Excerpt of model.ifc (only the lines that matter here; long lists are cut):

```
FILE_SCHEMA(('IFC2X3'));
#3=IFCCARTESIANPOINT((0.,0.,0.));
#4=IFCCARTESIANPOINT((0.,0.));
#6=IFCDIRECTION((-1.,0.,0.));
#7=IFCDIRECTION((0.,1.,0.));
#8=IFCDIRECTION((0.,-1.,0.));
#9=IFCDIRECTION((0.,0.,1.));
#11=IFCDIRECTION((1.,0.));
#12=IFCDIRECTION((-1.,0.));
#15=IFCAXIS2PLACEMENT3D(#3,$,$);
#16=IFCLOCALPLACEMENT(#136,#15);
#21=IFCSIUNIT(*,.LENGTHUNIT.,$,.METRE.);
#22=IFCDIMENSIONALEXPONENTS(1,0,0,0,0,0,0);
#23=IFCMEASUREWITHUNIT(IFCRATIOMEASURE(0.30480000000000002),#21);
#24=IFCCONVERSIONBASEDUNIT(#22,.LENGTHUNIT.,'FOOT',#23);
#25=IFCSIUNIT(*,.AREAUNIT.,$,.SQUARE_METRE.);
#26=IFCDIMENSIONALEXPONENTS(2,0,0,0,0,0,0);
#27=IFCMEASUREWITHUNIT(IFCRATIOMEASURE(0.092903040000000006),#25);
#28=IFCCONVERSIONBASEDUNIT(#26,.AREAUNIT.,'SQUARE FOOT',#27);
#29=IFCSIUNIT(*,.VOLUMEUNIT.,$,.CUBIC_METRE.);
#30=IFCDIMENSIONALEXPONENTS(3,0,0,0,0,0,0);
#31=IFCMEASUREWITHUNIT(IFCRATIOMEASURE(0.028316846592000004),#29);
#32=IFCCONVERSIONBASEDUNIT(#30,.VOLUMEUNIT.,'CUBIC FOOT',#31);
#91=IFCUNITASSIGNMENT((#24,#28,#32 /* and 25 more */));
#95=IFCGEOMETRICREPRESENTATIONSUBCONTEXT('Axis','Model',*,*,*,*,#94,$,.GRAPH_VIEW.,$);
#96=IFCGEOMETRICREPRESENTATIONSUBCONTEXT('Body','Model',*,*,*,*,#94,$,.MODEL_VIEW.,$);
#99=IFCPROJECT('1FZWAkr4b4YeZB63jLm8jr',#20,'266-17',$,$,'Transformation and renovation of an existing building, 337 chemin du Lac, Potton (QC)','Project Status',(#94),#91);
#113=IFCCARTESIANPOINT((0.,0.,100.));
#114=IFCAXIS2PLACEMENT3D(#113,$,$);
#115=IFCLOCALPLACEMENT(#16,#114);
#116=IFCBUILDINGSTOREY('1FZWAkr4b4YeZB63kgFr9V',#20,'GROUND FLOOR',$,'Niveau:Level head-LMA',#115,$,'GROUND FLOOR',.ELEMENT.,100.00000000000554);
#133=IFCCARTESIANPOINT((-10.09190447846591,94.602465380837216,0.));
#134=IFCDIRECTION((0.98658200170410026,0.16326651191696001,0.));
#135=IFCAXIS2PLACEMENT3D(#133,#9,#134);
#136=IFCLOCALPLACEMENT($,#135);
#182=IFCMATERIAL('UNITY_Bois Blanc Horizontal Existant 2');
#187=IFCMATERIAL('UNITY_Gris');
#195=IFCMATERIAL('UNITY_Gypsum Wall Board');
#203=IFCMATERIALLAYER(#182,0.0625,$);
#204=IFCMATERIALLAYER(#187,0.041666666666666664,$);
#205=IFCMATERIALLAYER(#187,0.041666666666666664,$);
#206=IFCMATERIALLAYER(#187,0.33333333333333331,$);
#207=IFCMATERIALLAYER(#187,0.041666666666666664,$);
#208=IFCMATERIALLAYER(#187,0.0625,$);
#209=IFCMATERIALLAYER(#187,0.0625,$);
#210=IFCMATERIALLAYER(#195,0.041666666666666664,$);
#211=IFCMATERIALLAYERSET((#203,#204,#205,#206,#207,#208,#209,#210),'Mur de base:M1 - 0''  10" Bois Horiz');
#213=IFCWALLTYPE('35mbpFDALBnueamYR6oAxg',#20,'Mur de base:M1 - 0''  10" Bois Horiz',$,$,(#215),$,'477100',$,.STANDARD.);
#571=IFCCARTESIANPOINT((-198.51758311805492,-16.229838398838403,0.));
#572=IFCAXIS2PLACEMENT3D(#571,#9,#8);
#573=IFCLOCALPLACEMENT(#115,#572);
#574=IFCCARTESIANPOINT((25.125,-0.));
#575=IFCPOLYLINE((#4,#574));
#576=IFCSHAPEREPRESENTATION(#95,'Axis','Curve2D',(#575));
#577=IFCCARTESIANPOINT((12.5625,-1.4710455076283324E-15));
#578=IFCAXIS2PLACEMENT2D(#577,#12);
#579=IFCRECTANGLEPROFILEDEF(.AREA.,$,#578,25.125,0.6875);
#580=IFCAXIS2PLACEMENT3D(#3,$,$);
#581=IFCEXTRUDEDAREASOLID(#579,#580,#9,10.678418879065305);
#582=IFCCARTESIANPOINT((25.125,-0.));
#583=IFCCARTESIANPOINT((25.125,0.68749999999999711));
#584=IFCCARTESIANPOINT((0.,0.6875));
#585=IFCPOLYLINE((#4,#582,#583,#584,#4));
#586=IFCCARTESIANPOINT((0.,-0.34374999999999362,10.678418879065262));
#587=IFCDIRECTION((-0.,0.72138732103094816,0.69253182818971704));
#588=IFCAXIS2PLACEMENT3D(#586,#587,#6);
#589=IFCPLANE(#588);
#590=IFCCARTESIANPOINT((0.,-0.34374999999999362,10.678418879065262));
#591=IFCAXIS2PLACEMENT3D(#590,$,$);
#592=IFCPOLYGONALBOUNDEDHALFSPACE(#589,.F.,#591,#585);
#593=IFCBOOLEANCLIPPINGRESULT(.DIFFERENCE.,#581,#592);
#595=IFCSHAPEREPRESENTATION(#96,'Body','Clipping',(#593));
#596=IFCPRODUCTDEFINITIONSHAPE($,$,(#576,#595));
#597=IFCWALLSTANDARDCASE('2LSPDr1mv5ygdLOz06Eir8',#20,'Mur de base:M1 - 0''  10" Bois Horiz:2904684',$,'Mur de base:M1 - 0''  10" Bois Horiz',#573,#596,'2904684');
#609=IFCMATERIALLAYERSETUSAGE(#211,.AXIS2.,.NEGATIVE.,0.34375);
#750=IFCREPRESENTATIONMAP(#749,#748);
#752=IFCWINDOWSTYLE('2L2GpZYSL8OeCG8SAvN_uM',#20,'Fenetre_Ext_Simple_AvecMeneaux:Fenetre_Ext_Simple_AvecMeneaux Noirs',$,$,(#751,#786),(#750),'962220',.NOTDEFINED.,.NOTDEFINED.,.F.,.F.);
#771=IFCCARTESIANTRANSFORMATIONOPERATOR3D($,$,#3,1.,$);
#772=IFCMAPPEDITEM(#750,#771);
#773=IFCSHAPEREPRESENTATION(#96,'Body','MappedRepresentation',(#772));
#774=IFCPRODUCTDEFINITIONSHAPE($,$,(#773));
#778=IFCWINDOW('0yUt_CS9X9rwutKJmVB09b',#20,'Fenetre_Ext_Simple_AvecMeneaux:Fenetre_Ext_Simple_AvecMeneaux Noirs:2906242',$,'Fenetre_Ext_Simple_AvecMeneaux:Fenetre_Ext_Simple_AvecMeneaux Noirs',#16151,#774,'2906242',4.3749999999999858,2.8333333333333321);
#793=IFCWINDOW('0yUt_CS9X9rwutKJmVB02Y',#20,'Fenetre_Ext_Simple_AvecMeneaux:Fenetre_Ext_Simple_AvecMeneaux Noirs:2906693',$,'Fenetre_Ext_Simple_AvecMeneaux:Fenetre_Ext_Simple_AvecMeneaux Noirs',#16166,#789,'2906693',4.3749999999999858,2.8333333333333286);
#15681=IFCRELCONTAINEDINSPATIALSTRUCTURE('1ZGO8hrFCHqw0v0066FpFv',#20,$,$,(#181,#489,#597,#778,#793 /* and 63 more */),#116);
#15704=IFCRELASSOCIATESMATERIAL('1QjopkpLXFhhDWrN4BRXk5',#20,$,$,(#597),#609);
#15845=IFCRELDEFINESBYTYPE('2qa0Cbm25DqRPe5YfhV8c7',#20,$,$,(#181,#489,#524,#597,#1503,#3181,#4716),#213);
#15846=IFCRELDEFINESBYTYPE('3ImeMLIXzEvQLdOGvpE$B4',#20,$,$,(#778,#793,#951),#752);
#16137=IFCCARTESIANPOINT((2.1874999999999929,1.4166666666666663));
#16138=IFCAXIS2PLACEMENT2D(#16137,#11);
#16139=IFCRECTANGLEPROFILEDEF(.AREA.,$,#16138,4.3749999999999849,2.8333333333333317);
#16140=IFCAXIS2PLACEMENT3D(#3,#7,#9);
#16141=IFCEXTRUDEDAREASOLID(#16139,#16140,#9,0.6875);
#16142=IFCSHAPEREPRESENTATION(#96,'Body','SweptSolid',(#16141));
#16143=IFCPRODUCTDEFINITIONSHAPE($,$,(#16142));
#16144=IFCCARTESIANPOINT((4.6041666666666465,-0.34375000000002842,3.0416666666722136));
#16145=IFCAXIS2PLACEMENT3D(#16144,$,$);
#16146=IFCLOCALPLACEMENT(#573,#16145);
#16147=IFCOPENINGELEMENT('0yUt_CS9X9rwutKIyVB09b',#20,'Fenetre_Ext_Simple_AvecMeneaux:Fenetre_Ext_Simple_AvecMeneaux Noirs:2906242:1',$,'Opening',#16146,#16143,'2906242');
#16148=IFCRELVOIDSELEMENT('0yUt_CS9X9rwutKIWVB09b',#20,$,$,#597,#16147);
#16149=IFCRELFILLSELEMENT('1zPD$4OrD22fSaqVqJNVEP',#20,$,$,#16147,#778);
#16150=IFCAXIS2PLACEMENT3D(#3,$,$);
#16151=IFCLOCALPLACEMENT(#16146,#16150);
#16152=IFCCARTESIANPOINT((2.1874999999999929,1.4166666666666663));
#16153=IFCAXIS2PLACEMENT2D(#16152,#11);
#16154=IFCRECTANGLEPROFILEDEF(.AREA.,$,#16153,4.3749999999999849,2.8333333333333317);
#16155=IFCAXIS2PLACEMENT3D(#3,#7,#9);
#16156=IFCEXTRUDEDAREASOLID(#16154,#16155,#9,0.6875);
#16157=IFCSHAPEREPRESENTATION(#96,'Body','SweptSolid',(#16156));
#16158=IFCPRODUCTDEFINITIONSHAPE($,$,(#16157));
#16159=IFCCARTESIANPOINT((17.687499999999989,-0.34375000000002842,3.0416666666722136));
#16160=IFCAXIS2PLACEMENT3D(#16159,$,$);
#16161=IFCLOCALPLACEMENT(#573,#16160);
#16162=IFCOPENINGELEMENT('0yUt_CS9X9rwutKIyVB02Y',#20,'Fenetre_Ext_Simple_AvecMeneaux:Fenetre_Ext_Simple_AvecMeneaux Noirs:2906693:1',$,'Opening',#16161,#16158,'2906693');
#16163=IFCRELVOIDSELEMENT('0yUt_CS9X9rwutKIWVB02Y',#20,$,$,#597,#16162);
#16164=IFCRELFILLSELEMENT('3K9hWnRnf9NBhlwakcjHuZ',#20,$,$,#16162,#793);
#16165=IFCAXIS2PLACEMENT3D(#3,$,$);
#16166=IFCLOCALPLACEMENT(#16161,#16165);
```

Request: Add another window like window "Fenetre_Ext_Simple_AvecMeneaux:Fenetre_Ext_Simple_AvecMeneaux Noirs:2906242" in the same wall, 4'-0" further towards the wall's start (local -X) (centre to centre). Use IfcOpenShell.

```python
import ifcopenshell
import ifcopenshell.api.feature
import ifcopenshell.api.geometry
import ifcopenshell.api.root
import ifcopenshell.geom
import ifcopenshell.util.element
import ifcopenshell.util.placement
import ifcopenshell.util.shape
import ifcopenshell.util.unit

model = ifcopenshell.open("model.ifc")
unit_scale = ifcopenshell.util.unit.calculate_unit_scale(model)
settings = ifcopenshell.geom.settings()


def volume(element):
    """Net volume in cubic metres, openings subtracted."""
    shape = ifcopenshell.geom.create_shape(settings, element)
    return ifcopenshell.util.shape.get_volume(shape.geometry)


def reuse_history(source, copy):
    """copy_class also copies each property set's owner history, people and application; keep the originals."""
    for rel in copy.IsDefinedBy:
        if rel.is_a("IfcRelDefinesByProperties") and (history := rel.RelatingPropertyDefinition.OwnerHistory):
            rel.RelatingPropertyDefinition.OwnerHistory = source.OwnerHistory
            ifcopenshell.util.element.remove_deep2(model, history)


window = model.by_guid("0yUt_CS9X9rwutKJmVB09b")
opening = window.FillsVoids[0].RelatingOpeningElement
wall = opening.VoidsElements[0].RelatingBuildingElement
before = volume(wall)
shift = ifcopenshell.util.placement.get_local_placement(wall.ObjectPlacement)[:3, 0] * -48 * 0.0254 / unit_scale

# copy_class copies the void relationship, type, container and properties, but no geometry.
new_opening = ifcopenshell.api.root.copy_class(model, product=opening)
new_opening.Representation = ifcopenshell.util.element.copy_deep(
    model, opening.Representation, exclude=["IfcGeometricRepresentationContext", "IfcRepresentationMap"]
)
new_opening.Name = "Fenetre_Ext_Simple_AvecMeneaux:Fenetre_Ext_Simple_AvecMeneaux Noirs"
new_opening.Tag = None
new_window = ifcopenshell.api.root.copy_class(model, product=window)
new_window.Representation = ifcopenshell.util.element.copy_deep(
    model, window.Representation, exclude=["IfcGeometricRepresentationContext", "IfcRepresentationMap"]
)
new_window.Name = "Fenetre_Ext_Simple_AvecMeneaux:Fenetre_Ext_Simple_AvecMeneaux Noirs"
new_window.Tag = None
reuse_history(window, new_window)
fills = ifcopenshell.api.feature.add_filling(model, opening=new_opening, element=new_window)
fills.OwnerHistory = new_window.OwnerHistory  # required in IFC2X3

for old, new in ((opening, new_opening), (window, new_window)):
    matrix = ifcopenshell.util.placement.get_local_placement(old.ObjectPlacement)
    matrix[:3, 3] += shift
    ifcopenshell.api.geometry.edit_object_placement(model, product=new, matrix=matrix, is_si=False)

after = volume(wall)

print(f"wall volume {before:.3f} -> {after:.3f} m3")

model.write("model_edited.ifc")
```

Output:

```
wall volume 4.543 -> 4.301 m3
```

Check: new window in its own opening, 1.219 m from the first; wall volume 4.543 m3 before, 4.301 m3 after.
